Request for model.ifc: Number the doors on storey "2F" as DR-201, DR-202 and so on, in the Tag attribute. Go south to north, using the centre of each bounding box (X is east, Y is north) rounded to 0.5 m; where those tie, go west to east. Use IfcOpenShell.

First a look at what the model holds.

```python
import ifcopenshell
import ifcopenshell.util.element
import ifcopenshell.util.placement

model = ifcopenshell.open("model.ifc")
print(model.schema)
storey = next(s for s in model.by_type("IfcBuildingStorey") if s.Name == "2F")
doors = [e for e in ifcopenshell.util.element.get_decomposition(storey) if e.is_a("IfcDoor")]
for e in sorted(doors, key=lambda e: e.id()):
    origin = ifcopenshell.util.placement.get_local_placement(e.ObjectPlacement)[:3, 3]
    print(e.id(), e.Tag, e.Name, origin.round(2) + 0.0, sep=" | ")
```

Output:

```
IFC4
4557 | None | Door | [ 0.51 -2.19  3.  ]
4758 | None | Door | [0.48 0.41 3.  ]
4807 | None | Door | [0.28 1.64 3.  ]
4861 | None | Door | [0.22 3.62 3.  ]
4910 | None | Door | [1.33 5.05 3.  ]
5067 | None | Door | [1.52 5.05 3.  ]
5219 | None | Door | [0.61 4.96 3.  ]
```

```python
import ifcopenshell
import ifcopenshell.geom
import ifcopenshell.util.element
import ifcopenshell.util.shape

model = ifcopenshell.open("model.ifc")
settings = ifcopenshell.geom.settings()
settings.set("use-world-coords", True)


def centre(element):
    shape = ifcopenshell.geom.create_shape(settings, element)
    return ifcopenshell.util.shape.get_bbox_centroid(shape.geometry)


storey = next(s for s in model.by_type("IfcBuildingStorey") if s.Name == "2F")
doors = [e for e in ifcopenshell.util.element.get_decomposition(storey) if e.is_a("IfcDoor")]

# Insertion points can sit at a corner or the storey origin, so sort by the geometry (in metres).
centres = {e: centre(e) for e in doors}
doors.sort(key=lambda e: (round(centres[e][1] / 0.5), centres[e][0]))

for i, e in enumerate(doors, start=1):
    number = f"DR-2{i:02d}"
    e.Tag = number
    print(e.id(), number)

model.write("model_updated.ifc")
```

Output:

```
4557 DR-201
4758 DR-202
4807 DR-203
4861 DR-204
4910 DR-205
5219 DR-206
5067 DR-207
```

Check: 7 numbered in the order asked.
